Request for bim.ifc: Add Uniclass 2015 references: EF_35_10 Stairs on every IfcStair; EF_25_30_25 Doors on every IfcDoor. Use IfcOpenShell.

First a look at what the model holds.

```python
import ifcopenshell

model = ifcopenshell.open("bim.ifc")
print(model.schema)
print("classifications:", [c.Name for c in model.by_type("IfcClassification")])
for ifc_class in ("IfcDoor", "IfcRoof", "IfcStair", "IfcWall", "IfcWindow"):
    print(ifc_class, len(model.by_type(ifc_class)))
```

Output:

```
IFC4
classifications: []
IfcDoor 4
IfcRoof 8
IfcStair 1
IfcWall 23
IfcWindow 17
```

```python
import ifcopenshell
import ifcopenshell.api.classification

model = ifcopenshell.open("bim.ifc")

system = ifcopenshell.api.classification.add_classification(model, classification="Uniclass 2015")

codes = {
    "IfcStair": ("EF_35_10", "Stairs"),
    "IfcDoor": ("EF_25_30_25", "Doors"),
}
for ifc_class, (code, name) in codes.items():
    products = model.by_type(ifc_class)
    ifcopenshell.api.classification.add_reference(
        model, products=products, classification=system, identification=code, name=name
    )
    print(code, len(products))

model.write("bim_rev.ifc")
```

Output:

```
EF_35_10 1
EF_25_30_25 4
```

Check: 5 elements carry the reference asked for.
